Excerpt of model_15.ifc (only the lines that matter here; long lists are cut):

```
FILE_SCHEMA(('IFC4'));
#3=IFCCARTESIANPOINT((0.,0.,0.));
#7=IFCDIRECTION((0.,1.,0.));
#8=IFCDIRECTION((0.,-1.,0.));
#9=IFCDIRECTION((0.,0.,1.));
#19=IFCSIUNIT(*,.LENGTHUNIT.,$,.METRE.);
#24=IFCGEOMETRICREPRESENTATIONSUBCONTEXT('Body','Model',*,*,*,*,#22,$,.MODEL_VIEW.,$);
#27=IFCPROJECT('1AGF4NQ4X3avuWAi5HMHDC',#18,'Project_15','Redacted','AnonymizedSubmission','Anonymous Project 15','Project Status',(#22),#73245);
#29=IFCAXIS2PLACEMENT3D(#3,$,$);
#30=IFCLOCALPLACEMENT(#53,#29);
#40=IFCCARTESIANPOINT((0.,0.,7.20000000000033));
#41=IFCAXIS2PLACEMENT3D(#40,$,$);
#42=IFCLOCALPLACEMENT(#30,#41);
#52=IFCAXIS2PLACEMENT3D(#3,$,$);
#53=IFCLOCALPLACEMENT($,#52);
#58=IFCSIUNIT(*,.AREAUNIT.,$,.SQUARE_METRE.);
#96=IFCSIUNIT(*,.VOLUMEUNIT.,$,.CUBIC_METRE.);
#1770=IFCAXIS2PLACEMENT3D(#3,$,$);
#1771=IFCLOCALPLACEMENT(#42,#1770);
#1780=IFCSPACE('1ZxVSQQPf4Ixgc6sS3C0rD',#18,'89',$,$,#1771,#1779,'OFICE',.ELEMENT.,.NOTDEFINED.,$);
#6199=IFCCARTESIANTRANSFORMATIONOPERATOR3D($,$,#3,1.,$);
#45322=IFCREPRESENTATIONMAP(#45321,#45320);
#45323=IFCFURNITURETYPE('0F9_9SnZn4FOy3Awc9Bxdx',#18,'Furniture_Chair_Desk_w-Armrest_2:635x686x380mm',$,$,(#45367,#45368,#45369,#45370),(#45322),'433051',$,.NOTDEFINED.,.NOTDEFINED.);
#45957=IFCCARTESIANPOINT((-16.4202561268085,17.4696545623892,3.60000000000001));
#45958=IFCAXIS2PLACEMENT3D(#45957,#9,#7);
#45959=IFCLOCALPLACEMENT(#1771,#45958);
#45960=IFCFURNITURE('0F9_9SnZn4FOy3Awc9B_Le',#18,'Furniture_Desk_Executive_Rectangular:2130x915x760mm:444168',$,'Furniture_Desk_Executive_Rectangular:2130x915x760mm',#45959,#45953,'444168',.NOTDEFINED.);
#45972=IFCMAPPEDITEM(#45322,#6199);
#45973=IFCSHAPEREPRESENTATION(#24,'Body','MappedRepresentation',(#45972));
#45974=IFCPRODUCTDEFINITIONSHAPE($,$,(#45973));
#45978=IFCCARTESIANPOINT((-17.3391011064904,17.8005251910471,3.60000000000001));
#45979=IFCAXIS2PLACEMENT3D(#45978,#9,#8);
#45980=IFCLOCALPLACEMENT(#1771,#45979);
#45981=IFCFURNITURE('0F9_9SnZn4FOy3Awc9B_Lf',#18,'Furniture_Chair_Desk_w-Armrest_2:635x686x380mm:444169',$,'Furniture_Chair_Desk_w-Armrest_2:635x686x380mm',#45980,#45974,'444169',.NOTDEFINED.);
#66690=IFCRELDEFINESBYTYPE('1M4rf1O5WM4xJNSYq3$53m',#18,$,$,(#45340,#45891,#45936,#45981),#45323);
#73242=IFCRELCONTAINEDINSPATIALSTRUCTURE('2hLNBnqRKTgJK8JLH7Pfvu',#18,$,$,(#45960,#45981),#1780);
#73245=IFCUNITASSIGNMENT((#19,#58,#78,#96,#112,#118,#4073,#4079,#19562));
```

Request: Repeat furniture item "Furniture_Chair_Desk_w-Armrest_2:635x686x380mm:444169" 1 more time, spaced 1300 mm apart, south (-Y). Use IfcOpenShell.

```python
import numpy as np
import ifcopenshell
import ifcopenshell.api.geometry
import ifcopenshell.api.root
import ifcopenshell.util.element
import ifcopenshell.util.placement

model = ifcopenshell.open("model_15.ifc")


def reuse_history(source, copy):
    """copy_class also copies each property set's owner history, people and application; keep the originals."""
    for rel in copy.IsDefinedBy:
        if rel.is_a("IfcRelDefinesByProperties") and (history := rel.RelatingPropertyDefinition.OwnerHistory):
            rel.RelatingPropertyDefinition.OwnerHistory = source.OwnerHistory
            ifcopenshell.util.element.remove_deep2(model, history)


source = model.by_guid("0F9_9SnZn4FOy3Awc9B_Lf")
base = ifcopenshell.util.placement.get_local_placement(source.ObjectPlacement)
step = np.array([0.0, -1.0, 0.0]) * 1.3

for i in range(1, 2):
    copy = ifcopenshell.api.root.copy_class(model, product=source)
    copy.Representation = ifcopenshell.util.element.copy_deep(
        model, source.Representation, exclude=["IfcGeometricRepresentationContext", "IfcRepresentationMap"]
    )
    copy.Name = "Furniture_Chair_Desk_w-Armrest_2:635x686x380mm"
    copy.Tag = None
    reuse_history(source, copy)
    matrix = base.copy()
    matrix[:3, 3] += i * step
    print("added at", matrix[:3, 3].round(3) + 0.0)
    ifcopenshell.api.geometry.edit_object_placement(model, product=copy, matrix=matrix, is_si=False)

model.write("model_15_edited.ifc")
```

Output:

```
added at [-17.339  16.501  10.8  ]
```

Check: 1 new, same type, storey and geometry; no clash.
